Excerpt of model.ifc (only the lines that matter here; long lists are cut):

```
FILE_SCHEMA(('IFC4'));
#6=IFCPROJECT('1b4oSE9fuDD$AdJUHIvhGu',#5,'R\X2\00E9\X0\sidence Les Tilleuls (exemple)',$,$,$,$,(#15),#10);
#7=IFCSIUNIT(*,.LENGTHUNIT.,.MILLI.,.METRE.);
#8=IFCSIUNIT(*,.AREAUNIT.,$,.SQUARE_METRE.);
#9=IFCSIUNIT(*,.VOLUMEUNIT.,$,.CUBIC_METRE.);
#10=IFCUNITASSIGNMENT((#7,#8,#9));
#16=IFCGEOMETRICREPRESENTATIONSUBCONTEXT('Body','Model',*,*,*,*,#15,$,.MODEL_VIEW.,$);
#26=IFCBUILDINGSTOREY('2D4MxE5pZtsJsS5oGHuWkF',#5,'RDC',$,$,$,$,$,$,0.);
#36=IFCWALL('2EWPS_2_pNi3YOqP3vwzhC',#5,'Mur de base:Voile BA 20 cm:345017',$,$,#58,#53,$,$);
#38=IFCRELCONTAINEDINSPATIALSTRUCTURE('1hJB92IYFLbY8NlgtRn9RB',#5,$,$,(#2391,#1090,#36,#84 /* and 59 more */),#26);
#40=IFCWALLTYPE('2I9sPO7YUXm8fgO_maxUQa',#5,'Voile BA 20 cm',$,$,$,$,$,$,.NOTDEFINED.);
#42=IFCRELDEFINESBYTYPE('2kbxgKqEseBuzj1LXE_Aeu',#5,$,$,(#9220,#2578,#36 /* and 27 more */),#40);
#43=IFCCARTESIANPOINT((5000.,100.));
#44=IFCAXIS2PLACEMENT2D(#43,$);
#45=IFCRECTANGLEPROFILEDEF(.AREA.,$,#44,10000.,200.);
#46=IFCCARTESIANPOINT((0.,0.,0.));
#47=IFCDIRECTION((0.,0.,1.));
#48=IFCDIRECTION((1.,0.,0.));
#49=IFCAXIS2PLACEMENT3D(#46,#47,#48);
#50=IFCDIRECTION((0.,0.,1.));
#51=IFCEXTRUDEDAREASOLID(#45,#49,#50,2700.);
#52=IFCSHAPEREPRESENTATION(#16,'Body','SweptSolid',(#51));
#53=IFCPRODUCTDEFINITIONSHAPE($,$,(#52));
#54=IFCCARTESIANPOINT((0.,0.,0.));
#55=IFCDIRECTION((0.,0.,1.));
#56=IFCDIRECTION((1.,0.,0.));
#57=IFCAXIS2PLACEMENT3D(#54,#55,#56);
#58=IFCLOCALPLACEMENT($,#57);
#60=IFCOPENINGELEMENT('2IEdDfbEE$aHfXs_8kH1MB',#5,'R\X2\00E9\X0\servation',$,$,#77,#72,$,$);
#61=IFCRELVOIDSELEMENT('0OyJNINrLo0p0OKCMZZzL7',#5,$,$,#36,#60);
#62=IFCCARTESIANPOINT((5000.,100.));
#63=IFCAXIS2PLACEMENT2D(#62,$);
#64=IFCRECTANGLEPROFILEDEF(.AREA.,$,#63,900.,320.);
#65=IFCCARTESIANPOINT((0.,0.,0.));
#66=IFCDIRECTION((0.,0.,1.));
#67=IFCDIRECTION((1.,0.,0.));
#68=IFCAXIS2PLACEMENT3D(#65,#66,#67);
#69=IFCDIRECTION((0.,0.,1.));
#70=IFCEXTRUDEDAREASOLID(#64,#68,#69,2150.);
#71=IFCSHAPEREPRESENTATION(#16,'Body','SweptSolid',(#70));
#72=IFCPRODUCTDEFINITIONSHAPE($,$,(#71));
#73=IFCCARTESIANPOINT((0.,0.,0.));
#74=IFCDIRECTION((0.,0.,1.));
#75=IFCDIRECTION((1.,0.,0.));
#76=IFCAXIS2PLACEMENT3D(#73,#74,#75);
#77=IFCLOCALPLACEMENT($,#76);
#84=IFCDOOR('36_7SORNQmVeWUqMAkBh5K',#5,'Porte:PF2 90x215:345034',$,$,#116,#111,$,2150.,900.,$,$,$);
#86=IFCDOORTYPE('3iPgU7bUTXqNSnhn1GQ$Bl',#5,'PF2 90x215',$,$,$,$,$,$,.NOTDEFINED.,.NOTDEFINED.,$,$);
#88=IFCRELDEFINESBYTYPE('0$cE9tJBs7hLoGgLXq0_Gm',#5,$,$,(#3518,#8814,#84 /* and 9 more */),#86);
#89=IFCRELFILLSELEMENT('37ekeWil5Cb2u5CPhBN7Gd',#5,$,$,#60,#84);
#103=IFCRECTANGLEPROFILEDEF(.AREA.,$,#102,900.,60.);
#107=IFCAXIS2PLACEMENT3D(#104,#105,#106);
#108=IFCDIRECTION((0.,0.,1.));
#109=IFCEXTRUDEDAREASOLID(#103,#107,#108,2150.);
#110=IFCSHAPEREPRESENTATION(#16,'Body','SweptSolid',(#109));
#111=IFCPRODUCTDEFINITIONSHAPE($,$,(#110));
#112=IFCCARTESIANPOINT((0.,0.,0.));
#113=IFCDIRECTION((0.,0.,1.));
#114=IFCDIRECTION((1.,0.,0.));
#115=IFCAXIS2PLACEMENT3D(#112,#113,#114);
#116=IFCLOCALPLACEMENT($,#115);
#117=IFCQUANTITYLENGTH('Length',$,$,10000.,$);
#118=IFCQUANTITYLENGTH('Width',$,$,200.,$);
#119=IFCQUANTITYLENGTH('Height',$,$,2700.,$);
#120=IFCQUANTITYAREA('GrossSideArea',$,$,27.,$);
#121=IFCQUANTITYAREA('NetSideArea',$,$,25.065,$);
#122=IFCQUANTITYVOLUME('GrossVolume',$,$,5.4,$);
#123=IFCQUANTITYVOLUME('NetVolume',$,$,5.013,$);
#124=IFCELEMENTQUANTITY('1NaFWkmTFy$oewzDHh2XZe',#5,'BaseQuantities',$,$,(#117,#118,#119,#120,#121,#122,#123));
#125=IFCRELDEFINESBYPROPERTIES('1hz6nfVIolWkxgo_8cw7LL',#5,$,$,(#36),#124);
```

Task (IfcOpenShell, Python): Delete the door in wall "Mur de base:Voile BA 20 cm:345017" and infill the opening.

```python
import ifcopenshell
import ifcopenshell.api.feature
import ifcopenshell.api.pset
import ifcopenshell.api.root
import ifcopenshell.geom
import ifcopenshell.util.element
import ifcopenshell.util.shape
import ifcopenshell.util.unit

model = ifcopenshell.open("model.ifc")
area_scale = ifcopenshell.util.unit.calculate_unit_scale(model, "AREAUNIT")
volume_scale = ifcopenshell.util.unit.calculate_unit_scale(model, "VOLUMEUNIT")
settings = ifcopenshell.geom.settings()


def volume(element):
    """Net volume in cubic metres, openings subtracted."""
    shape = ifcopenshell.geom.create_shape(settings, element)
    return ifcopenshell.util.shape.get_volume(shape.geometry)


door = model.by_guid("36_7SORNQmVeWUqMAkBh5K")
opening = door.FillsVoids[0].RelatingOpeningElement
wall = opening.VoidsElements[0].RelatingBuildingElement
before = volume(wall)

ifcopenshell.api.root.remove_product(model, product=door)
ifcopenshell.api.feature.remove_feature(model, feature=opening)

after = volume(wall)
thickness = 0.2  # wall thickness in metres

# Update the wall's stored quantities.
qto = model.by_id(ifcopenshell.util.element.get_pset(wall, "BaseQuantities", should_inherit=False)["id"])
ifcopenshell.api.pset.edit_qto(model, qto=qto, properties={
    "NetSideArea": after / thickness / area_scale,
    "NetVolume": after / volume_scale,
})

print(f"wall volume {before:.3f} -> {after:.3f} m3")

model.write("model_edited.ifc")
```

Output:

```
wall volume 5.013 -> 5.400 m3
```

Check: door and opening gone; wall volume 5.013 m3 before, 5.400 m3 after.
